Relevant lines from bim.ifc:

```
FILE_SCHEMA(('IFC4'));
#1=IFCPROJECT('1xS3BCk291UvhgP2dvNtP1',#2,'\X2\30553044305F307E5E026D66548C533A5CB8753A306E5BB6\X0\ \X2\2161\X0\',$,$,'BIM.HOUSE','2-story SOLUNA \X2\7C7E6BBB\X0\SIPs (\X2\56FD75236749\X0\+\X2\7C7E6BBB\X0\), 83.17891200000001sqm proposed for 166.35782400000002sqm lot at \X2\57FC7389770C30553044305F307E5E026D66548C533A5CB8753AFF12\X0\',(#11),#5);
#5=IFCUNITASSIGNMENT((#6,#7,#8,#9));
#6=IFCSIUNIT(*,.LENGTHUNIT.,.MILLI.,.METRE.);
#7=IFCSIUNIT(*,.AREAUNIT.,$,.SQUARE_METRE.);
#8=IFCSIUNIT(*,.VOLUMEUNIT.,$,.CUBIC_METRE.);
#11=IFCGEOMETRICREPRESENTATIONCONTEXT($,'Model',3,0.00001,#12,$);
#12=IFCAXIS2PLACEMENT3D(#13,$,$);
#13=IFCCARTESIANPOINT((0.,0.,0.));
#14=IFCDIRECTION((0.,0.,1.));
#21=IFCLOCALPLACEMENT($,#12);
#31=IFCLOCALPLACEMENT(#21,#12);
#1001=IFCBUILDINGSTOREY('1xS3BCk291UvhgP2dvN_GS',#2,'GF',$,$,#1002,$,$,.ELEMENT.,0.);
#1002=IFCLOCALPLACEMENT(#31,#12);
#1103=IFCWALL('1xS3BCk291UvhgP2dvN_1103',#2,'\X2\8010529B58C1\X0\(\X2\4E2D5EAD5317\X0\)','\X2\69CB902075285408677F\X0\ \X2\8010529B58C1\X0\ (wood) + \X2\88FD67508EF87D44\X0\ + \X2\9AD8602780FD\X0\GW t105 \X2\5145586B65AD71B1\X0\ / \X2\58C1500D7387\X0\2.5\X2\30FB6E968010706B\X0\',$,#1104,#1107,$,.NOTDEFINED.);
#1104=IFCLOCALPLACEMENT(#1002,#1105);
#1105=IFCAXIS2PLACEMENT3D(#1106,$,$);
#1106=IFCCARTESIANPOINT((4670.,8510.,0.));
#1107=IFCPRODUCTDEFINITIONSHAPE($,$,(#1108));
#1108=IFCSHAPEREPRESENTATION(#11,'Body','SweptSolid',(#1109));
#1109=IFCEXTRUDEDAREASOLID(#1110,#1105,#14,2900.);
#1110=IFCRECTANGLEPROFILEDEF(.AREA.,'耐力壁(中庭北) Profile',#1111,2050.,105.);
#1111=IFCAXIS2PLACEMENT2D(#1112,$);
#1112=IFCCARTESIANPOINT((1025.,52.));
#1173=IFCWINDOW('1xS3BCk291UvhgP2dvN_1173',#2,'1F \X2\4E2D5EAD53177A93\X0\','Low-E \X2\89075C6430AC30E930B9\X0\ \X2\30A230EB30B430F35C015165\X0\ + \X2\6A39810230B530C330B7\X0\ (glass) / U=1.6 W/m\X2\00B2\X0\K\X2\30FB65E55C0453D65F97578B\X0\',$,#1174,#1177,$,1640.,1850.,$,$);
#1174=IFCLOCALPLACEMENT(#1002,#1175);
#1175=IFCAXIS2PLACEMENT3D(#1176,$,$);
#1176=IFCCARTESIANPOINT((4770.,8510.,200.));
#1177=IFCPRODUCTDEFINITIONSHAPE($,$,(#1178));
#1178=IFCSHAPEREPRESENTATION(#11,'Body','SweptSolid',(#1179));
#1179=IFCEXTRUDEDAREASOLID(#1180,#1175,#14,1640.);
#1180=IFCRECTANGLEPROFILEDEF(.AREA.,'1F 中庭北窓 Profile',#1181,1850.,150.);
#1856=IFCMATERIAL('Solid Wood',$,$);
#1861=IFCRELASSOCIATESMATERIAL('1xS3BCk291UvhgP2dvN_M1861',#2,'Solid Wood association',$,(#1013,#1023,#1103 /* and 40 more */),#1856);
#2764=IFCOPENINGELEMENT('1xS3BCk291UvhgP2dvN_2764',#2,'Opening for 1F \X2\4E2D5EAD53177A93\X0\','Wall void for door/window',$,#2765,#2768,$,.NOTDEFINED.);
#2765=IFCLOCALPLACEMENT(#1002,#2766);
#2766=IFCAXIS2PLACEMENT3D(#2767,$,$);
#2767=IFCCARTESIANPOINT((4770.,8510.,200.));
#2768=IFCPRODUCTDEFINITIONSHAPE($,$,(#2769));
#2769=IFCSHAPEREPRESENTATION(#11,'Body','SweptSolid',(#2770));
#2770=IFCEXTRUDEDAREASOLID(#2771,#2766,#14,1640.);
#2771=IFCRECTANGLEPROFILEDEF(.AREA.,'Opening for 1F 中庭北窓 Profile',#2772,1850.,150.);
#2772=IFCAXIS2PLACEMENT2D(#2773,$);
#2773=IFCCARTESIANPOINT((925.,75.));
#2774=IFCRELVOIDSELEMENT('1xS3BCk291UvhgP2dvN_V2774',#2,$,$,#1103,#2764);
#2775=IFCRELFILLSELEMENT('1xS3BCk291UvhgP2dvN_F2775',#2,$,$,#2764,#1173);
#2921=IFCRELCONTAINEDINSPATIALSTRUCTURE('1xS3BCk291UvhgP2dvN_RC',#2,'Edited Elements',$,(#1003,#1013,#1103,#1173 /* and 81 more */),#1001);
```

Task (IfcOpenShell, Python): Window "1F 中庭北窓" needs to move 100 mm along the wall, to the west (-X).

```python
import ifcopenshell
import ifcopenshell.api.geometry
import ifcopenshell.util.placement
import ifcopenshell.util.unit

model = ifcopenshell.open("bim.ifc")
unit_scale = ifcopenshell.util.unit.calculate_unit_scale(model)

window = model.by_guid("1xS3BCk291UvhgP2dvN_1173")
opening = window.FillsVoids[0].RelatingOpeningElement
wall = opening.VoidsElements[0].RelatingBuildingElement

wall_matrix = ifcopenshell.util.placement.get_local_placement(wall.ObjectPlacement)
shift = wall_matrix[:3, 0] * -0.1 / unit_scale
before = ifcopenshell.util.placement.get_local_placement(window.ObjectPlacement)[:3, 3].copy()

# The window is not placed relative to its opening, so move both.
for product in (opening, window):
    matrix = ifcopenshell.util.placement.get_local_placement(product.ObjectPlacement)
    matrix[:3, 3] += shift
    ifcopenshell.api.geometry.edit_object_placement(model, product=product, matrix=matrix, is_si=False)

after = ifcopenshell.util.placement.get_local_placement(window.ObjectPlacement)[:3, 3]
print("window moved by", (after - before).round(3) + 0.0)

model.write("bim_v2.ifc")
```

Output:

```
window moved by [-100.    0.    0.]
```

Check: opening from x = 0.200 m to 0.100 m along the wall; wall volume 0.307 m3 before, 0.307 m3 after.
